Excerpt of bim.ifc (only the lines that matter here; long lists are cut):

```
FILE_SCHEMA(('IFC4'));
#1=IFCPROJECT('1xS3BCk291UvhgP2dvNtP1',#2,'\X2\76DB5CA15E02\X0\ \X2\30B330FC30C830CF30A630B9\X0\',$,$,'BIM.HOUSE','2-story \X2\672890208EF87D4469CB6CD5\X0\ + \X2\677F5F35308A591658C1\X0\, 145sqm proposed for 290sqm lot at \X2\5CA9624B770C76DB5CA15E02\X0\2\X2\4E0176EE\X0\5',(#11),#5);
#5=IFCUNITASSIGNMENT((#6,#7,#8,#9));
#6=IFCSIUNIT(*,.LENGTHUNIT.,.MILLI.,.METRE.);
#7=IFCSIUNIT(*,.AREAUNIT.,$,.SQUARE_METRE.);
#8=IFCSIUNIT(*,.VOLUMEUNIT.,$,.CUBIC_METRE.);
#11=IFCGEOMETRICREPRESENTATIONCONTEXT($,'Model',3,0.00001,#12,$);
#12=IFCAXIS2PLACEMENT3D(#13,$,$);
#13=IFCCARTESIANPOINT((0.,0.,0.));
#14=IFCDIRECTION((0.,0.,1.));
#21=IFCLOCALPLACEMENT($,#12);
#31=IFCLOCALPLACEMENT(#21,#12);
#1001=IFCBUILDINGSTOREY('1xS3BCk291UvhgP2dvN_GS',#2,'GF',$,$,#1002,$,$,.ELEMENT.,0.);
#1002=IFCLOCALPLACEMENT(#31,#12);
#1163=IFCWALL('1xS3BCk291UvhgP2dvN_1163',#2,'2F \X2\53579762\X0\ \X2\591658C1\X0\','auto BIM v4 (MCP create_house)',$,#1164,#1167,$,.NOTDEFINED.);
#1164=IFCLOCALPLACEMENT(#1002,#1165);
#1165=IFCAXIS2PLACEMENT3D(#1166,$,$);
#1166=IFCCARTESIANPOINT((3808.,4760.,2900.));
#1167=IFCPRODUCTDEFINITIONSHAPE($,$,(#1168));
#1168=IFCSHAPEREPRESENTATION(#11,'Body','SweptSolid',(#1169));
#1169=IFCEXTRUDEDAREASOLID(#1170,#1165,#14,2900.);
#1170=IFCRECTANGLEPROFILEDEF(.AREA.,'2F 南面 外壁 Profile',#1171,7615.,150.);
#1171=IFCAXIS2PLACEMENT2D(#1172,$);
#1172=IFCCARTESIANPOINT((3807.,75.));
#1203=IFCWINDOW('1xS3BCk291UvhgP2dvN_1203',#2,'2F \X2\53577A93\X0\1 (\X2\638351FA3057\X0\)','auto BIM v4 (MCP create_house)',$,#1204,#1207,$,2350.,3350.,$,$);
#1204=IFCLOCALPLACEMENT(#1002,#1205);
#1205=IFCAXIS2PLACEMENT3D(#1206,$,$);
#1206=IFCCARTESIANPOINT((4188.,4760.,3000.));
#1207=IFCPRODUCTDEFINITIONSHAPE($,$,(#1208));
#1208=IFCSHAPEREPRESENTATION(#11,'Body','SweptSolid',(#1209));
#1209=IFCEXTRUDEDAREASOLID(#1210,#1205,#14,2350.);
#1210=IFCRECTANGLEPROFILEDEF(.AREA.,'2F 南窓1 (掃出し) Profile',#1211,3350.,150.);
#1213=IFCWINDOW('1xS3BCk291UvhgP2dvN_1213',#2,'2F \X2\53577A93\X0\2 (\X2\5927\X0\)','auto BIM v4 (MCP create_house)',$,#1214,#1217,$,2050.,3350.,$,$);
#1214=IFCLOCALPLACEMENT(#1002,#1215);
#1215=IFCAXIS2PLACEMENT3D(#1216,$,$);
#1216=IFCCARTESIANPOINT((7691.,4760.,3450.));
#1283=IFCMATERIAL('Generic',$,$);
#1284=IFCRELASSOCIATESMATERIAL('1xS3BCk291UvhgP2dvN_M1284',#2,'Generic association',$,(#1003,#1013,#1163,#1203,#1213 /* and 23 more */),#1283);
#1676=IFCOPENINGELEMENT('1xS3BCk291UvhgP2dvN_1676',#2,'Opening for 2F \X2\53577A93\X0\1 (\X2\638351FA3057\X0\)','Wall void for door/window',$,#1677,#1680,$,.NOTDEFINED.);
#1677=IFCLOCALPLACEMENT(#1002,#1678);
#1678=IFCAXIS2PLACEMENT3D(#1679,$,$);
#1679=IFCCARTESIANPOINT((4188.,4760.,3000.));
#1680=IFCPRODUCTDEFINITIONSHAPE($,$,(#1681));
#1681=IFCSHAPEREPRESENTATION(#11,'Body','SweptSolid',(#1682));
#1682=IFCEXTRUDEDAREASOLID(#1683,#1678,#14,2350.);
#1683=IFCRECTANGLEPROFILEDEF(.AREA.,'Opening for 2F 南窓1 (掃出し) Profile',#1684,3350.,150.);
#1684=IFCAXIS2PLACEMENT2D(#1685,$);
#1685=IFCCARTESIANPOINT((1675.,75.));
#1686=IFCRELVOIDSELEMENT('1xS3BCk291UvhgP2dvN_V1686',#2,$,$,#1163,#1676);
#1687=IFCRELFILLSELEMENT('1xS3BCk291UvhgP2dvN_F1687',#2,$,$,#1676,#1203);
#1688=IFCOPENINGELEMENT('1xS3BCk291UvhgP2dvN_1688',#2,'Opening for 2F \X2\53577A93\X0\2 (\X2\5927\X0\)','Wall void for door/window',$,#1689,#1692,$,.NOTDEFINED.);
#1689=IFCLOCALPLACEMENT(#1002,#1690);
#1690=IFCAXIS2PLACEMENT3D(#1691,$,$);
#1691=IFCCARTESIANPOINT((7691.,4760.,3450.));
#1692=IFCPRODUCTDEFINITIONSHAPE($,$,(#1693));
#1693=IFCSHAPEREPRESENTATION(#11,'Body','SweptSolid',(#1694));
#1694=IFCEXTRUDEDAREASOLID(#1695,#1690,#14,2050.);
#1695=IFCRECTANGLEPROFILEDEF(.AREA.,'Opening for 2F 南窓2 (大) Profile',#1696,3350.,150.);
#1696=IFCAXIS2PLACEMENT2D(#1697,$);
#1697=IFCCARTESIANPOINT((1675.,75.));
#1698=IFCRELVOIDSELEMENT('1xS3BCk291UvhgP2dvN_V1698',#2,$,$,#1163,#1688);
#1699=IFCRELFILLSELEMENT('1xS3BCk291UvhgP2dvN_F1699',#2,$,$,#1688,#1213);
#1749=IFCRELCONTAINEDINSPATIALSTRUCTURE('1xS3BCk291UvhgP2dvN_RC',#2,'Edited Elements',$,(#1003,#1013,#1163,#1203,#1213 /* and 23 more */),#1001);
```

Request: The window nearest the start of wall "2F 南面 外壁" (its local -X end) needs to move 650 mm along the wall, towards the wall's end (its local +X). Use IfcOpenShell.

```python
import ifcopenshell
import ifcopenshell.api.geometry
import ifcopenshell.util.placement

model = ifcopenshell.open("bim.ifc")

window = model.by_guid("1xS3BCk291UvhgP2dvN_1203")
opening = window.FillsVoids[0].RelatingOpeningElement
wall = opening.VoidsElements[0].RelatingBuildingElement

wall_matrix = ifcopenshell.util.placement.get_local_placement(wall.ObjectPlacement)
shift = wall_matrix[:3, 0] * 650.0
before = ifcopenshell.util.placement.get_local_placement(window.ObjectPlacement)[:3, 3].copy()

# The window is not placed relative to its opening, so move both.
for product in (opening, window):
    matrix = ifcopenshell.util.placement.get_local_placement(product.ObjectPlacement)
    matrix[:3, 3] += shift
    ifcopenshell.api.geometry.edit_object_placement(model, product=product, matrix=matrix, is_si=False)

after = ifcopenshell.util.placement.get_local_placement(window.ObjectPlacement)[:3, 3]
print("window moved by", (after - before).round(3) + 0.0)

model.write("bim_updated.ifc")
```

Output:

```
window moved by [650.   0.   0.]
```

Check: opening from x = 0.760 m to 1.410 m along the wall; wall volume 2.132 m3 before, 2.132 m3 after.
